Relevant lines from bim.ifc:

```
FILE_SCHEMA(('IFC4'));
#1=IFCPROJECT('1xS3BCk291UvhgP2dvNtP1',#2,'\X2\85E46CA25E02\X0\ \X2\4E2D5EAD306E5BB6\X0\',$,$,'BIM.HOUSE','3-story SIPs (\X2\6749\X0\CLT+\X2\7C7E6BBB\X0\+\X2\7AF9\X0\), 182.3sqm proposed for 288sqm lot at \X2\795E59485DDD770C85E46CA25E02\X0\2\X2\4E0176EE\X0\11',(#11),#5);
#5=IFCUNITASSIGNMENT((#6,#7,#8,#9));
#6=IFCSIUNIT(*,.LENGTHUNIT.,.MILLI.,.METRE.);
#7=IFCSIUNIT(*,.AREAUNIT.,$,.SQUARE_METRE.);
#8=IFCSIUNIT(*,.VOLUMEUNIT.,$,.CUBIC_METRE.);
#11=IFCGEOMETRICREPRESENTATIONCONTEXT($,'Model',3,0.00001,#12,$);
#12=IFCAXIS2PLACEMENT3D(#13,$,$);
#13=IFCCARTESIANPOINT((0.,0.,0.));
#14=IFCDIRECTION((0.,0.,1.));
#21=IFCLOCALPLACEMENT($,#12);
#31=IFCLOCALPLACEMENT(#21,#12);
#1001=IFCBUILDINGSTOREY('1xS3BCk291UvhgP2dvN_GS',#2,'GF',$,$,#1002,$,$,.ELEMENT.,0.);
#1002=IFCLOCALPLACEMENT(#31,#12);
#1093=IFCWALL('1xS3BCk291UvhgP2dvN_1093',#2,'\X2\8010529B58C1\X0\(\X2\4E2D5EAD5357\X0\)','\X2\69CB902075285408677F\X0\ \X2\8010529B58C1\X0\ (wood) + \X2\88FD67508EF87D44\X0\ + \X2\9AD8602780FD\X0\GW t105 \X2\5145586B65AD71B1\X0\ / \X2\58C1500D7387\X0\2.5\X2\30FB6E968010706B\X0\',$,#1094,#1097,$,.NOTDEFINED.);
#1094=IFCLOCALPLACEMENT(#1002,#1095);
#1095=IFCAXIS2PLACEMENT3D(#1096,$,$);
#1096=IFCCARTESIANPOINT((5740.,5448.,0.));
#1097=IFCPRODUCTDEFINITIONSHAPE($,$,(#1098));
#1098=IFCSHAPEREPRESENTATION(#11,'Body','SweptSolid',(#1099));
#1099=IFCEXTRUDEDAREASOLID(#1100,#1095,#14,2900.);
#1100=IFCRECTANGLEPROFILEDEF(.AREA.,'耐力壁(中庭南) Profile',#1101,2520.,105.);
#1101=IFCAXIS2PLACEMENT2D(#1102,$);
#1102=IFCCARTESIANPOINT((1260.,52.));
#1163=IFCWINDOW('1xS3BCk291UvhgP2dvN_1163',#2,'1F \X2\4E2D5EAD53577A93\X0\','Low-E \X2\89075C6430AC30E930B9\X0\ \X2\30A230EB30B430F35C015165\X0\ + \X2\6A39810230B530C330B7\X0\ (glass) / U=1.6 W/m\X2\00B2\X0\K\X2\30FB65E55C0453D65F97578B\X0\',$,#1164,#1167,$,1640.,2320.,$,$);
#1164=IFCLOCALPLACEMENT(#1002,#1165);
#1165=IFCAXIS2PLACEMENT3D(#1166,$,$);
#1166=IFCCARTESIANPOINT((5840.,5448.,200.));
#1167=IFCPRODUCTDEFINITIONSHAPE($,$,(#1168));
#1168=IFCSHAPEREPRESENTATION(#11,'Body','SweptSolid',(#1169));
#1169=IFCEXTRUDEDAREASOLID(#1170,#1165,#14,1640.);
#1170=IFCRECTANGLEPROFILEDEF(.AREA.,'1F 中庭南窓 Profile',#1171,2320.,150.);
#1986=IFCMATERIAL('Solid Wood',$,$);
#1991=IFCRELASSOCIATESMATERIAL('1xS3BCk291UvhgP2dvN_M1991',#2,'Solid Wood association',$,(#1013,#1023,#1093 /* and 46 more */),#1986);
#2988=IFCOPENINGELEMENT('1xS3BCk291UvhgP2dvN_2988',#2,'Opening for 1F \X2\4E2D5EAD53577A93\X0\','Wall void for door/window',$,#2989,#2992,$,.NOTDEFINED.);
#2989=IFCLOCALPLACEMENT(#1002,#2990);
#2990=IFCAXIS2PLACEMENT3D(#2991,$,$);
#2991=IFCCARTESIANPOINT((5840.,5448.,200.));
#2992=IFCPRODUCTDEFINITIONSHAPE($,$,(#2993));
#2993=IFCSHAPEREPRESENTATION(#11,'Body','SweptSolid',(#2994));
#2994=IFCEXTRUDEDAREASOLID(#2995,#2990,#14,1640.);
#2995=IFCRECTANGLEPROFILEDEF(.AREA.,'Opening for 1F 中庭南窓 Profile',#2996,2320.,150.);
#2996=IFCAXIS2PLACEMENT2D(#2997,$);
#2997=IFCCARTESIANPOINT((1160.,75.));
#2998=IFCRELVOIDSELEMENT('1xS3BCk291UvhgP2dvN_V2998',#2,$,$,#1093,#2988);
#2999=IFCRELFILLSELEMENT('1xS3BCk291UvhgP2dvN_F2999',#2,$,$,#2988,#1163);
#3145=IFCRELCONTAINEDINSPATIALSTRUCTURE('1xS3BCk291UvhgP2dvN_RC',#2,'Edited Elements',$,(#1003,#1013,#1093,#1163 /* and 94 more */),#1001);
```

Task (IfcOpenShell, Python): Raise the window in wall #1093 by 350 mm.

```python
import numpy as np
import ifcopenshell
import ifcopenshell.api.geometry
import ifcopenshell.util.placement
import ifcopenshell.util.unit

model = ifcopenshell.open("bim.ifc")
unit_scale = ifcopenshell.util.unit.calculate_unit_scale(model)

window = model.by_guid("1xS3BCk291UvhgP2dvN_1163")
opening = window.FillsVoids[0].RelatingOpeningElement
dz = 0.35 / unit_scale

shift = np.array([0.0, 0.0, dz])
# The window is not placed relative to its opening, so move both.
for product in (opening, window):
    matrix = ifcopenshell.util.placement.get_local_placement(product.ObjectPlacement)
    matrix[:3, 3] += shift
    ifcopenshell.api.geometry.edit_object_placement(model, product=product, matrix=matrix, is_si=False)

print(f"moved by {dz * unit_scale:+.3f} m")

model.write("bim_rev.ifc")
```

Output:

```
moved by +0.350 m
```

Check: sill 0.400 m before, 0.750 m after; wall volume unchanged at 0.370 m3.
